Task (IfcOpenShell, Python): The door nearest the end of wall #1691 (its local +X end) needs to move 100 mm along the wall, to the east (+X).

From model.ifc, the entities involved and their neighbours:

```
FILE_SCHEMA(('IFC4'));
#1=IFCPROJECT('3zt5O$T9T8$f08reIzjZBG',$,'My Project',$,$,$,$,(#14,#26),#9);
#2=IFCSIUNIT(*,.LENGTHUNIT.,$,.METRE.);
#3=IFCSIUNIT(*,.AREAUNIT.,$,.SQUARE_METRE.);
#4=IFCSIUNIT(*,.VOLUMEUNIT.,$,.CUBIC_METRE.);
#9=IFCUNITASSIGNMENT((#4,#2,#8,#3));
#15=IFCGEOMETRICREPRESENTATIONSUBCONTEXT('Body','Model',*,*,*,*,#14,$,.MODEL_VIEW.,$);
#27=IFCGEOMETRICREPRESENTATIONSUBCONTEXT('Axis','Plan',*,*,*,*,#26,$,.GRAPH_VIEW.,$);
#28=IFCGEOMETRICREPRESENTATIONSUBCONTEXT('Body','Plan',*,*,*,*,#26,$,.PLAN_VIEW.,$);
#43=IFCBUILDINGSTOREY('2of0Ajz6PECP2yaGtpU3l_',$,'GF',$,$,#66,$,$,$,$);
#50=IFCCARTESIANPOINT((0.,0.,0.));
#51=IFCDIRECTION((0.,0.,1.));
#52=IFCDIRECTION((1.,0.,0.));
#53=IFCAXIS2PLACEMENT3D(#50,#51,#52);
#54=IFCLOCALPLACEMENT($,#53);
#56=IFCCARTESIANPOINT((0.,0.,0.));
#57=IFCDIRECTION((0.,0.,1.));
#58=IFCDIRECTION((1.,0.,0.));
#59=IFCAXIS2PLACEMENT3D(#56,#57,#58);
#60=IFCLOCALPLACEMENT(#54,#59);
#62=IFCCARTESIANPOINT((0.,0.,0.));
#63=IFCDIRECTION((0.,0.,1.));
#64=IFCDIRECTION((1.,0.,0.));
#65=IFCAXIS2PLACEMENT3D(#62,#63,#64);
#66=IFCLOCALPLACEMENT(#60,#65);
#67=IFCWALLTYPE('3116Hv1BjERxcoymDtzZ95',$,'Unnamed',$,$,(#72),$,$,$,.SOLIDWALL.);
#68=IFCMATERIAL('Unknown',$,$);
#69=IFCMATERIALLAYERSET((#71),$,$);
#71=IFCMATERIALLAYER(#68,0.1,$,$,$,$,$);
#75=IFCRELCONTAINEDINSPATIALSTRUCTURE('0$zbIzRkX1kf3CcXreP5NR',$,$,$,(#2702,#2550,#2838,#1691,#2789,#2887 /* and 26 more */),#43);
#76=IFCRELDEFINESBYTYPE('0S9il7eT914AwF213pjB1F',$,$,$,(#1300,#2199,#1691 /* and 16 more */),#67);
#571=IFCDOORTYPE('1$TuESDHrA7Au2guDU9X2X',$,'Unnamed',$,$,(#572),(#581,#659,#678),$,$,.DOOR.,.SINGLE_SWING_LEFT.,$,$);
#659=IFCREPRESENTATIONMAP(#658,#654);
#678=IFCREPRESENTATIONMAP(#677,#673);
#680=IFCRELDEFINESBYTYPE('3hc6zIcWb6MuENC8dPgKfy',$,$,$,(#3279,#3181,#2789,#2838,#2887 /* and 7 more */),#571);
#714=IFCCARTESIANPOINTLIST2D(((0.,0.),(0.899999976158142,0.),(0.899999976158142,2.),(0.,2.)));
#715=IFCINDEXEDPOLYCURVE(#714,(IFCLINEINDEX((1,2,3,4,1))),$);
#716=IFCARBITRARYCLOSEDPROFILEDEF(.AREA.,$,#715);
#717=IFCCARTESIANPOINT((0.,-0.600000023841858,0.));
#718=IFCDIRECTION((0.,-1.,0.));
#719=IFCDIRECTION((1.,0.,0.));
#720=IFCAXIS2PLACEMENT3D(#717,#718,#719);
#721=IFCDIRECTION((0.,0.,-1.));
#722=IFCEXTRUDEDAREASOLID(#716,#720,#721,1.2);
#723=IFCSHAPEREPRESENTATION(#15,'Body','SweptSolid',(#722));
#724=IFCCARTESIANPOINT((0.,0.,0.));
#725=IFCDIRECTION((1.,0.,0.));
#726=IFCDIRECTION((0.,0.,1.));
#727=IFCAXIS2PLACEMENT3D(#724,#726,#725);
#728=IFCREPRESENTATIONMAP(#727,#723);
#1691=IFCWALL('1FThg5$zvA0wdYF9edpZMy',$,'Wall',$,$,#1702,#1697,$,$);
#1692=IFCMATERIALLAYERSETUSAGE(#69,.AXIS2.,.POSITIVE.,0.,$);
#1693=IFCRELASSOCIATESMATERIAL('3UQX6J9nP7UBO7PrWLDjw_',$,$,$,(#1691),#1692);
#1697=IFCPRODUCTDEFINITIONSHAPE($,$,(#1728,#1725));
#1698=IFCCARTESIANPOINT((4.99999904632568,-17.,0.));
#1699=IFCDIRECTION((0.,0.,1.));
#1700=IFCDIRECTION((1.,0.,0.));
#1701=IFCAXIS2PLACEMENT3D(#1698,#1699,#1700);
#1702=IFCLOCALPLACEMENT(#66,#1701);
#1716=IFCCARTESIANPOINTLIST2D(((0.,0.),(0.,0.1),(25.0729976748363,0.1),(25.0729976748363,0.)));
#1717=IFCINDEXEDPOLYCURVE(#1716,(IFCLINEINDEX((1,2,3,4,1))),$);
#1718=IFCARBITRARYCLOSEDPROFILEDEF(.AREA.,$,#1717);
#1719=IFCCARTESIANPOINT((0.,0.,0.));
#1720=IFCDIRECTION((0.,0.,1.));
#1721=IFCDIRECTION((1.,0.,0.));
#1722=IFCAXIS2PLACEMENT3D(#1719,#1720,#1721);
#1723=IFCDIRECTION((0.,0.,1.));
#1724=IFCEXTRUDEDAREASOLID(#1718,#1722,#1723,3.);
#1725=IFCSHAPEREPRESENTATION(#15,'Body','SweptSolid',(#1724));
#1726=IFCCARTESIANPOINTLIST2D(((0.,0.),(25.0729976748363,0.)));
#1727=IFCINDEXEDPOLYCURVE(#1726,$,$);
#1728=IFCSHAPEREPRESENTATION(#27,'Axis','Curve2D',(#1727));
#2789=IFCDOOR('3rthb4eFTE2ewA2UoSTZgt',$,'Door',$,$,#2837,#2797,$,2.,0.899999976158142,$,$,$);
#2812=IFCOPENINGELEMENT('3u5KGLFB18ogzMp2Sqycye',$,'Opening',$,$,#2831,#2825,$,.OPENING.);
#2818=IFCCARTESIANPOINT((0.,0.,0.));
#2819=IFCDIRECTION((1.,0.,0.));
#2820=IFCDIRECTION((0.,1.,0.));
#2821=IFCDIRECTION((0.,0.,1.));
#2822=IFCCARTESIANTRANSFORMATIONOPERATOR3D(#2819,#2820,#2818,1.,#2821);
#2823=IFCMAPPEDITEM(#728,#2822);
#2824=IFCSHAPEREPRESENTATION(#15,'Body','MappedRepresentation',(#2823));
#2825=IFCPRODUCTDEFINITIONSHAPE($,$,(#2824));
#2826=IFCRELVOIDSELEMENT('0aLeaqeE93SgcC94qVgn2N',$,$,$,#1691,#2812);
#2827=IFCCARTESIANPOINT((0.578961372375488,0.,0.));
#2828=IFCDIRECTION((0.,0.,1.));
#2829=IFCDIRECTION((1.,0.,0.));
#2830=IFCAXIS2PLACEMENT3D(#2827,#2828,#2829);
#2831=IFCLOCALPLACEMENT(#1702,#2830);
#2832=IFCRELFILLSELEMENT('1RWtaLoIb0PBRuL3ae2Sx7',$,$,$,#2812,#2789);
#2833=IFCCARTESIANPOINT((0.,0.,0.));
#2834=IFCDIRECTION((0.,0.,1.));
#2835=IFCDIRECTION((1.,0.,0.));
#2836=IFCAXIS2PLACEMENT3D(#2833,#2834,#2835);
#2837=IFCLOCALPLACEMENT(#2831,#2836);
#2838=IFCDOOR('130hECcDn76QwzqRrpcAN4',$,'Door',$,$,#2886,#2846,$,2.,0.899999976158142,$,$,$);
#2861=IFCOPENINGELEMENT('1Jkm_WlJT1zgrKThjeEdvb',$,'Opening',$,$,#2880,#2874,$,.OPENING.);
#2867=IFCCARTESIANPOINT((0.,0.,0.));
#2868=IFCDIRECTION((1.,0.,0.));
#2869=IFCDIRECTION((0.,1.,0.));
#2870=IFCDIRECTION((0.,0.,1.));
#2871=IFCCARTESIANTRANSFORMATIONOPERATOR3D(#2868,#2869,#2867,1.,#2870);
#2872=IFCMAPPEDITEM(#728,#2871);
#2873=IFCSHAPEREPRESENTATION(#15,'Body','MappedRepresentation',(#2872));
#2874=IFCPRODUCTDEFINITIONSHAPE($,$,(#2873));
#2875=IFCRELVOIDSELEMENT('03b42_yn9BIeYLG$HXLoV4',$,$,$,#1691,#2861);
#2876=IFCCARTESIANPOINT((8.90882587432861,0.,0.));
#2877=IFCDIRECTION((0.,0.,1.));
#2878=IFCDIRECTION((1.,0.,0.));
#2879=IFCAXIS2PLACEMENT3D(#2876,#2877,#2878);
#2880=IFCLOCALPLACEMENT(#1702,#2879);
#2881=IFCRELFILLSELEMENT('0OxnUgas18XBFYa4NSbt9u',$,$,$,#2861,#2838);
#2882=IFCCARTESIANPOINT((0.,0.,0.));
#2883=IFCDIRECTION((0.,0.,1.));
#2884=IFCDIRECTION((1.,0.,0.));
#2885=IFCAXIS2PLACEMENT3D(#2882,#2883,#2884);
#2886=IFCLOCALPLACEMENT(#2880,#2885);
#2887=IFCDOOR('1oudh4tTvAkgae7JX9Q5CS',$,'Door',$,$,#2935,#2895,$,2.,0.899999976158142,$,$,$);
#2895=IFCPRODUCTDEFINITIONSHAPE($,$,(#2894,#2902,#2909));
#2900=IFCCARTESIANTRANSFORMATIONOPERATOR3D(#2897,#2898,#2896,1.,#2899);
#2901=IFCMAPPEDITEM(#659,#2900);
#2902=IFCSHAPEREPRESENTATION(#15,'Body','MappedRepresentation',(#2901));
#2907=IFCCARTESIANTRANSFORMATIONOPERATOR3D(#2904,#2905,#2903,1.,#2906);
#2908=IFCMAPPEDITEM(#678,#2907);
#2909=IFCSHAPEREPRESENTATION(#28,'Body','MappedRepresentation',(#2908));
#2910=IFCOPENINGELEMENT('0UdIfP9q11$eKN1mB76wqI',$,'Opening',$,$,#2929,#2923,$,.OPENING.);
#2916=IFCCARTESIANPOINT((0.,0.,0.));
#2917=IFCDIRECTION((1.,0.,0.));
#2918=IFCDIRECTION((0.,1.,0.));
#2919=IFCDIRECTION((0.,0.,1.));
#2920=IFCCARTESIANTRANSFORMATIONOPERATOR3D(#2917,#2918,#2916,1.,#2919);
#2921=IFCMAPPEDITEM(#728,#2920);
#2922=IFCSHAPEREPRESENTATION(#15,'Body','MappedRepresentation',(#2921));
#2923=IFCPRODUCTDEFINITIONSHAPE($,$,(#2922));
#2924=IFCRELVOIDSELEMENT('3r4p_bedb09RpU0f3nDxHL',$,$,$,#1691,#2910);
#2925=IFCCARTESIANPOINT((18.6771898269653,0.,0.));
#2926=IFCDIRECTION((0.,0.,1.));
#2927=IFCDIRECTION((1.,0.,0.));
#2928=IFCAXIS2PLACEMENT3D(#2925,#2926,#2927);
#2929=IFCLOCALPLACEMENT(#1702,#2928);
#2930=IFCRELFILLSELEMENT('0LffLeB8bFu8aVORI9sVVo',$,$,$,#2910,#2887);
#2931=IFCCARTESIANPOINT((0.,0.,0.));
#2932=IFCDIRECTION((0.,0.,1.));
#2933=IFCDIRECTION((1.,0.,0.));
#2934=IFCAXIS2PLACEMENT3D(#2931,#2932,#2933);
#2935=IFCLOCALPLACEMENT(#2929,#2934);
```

```python
import ifcopenshell
import ifcopenshell.api.geometry
import ifcopenshell.util.placement

model = ifcopenshell.open("model.ifc")

door = model.by_guid("1oudh4tTvAkgae7JX9Q5CS")
opening = door.FillsVoids[0].RelatingOpeningElement
wall = opening.VoidsElements[0].RelatingBuildingElement

wall_matrix = ifcopenshell.util.placement.get_local_placement(wall.ObjectPlacement)
shift = wall_matrix[:3, 0] * 0.1
before = ifcopenshell.util.placement.get_local_placement(door.ObjectPlacement)[:3, 3].copy()

# The door is placed relative to its opening, so it follows when the opening moves.
matrix = ifcopenshell.util.placement.get_local_placement(opening.ObjectPlacement)
matrix[:3, 3] += shift
ifcopenshell.api.geometry.edit_object_placement(
    model, product=opening, matrix=matrix, is_si=False, should_transform_children=True
)

after = ifcopenshell.util.placement.get_local_placement(door.ObjectPlacement)[:3, 3]
print("door moved by", (after - before).round(3) + 0.0)

model.write("model_v2.ifc")
```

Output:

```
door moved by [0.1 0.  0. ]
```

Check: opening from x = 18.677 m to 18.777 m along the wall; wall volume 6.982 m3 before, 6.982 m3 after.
